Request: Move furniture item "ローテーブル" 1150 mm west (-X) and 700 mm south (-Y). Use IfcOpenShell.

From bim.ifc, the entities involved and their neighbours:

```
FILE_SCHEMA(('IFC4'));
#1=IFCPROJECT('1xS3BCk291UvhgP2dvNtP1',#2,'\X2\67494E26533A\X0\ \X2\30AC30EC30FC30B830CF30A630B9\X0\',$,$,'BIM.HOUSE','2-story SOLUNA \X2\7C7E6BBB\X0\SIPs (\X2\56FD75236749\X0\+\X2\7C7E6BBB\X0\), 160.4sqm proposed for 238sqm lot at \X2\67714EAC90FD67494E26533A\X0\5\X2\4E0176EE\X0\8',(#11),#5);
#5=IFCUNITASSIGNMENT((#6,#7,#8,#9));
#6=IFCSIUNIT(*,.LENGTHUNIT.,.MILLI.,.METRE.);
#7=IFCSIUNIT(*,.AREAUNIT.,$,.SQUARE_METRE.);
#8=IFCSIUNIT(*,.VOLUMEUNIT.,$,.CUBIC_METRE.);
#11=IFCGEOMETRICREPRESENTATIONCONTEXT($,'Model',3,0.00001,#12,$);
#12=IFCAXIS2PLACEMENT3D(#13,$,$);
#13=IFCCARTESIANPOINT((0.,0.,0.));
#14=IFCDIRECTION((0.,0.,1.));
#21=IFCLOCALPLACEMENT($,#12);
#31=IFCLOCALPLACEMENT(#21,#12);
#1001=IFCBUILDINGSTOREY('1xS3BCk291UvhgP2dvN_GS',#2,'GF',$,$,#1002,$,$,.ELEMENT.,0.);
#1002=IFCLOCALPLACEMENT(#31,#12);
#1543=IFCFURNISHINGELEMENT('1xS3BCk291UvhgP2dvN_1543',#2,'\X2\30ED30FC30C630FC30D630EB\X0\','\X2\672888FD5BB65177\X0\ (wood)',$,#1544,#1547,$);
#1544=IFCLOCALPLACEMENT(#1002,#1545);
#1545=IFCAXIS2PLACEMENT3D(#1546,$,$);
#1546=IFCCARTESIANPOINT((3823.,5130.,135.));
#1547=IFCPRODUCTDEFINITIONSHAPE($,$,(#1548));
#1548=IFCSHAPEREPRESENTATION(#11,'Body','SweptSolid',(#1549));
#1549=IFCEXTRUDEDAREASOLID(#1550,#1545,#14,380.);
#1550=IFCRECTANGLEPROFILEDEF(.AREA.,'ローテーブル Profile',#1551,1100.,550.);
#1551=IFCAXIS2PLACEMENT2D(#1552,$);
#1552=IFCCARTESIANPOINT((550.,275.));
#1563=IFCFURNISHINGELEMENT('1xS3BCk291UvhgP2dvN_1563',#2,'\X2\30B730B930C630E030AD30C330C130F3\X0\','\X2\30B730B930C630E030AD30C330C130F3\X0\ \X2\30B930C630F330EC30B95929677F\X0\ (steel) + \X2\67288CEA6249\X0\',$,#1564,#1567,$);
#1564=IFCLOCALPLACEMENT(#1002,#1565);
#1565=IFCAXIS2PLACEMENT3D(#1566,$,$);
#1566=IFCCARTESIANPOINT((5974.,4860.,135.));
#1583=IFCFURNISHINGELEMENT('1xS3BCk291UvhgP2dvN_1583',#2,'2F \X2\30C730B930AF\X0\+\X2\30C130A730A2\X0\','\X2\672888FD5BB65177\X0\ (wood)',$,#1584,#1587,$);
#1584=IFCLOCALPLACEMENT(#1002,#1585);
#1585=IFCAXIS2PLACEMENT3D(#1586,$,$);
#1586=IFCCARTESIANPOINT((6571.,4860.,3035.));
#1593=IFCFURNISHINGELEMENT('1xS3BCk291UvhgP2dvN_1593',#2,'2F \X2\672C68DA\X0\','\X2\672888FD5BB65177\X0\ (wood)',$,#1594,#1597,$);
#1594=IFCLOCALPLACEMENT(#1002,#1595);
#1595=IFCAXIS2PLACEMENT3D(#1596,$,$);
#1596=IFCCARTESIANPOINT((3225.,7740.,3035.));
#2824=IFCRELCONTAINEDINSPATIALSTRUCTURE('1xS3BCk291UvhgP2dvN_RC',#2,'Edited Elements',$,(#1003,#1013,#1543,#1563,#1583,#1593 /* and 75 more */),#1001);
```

```python
import ifcopenshell
import ifcopenshell.api.geometry
import ifcopenshell.util.placement
import ifcopenshell.util.unit

model = ifcopenshell.open("bim.ifc")
unit_scale = ifcopenshell.util.unit.calculate_unit_scale(model)

item = model.by_id(1543)
matrix = ifcopenshell.util.placement.get_local_placement(item.ObjectPlacement)
matrix[0, 3] -= 1.15 / unit_scale
matrix[1, 3] -= 0.7 / unit_scale
ifcopenshell.api.geometry.edit_object_placement(model, product=item, matrix=matrix, is_si=False)

print(ifcopenshell.util.placement.get_local_placement(item.ObjectPlacement).round(3) + 0.0)

model.write("bim-out.ifc")
```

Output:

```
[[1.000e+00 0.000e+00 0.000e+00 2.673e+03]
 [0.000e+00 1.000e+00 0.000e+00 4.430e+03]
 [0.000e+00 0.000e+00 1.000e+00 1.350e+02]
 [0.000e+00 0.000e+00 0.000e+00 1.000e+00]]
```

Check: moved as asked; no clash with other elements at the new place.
